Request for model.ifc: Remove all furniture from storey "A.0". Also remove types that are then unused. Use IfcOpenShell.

First a look at what the model holds.

```python
import ifcopenshell
import ifcopenshell.util.element

model = ifcopenshell.open("model.ifc")
print(model.schema)
storey = next(s for s in model.by_type("IfcBuildingStorey") if s.Name == "A.0")
furniture = [e for e in ifcopenshell.util.element.get_decomposition(storey) if e.is_a("IfcFurnishingElement")]
seen = {}
for e in furniture:
    element_type = ifcopenshell.util.element.get_type(e)
    name = element_type.Name if element_type not in (None, e) else None
    seen[name] = seen.get(name, 0) + 1
for name, count in sorted(seen.items(), key=str):
    print(count, "x", name)
```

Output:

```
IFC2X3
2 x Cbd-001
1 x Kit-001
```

```python
import ifcopenshell
import ifcopenshell.api.root
import ifcopenshell.util.element

model = ifcopenshell.open("model.ifc")

storey = next(s for s in model.by_type("IfcBuildingStorey") if s.Name == "A.0")
furniture = [e for e in ifcopenshell.util.element.get_decomposition(storey) if e.is_a("IfcFurnishingElement")]
types = {ifcopenshell.util.element.get_type(e) for e in furniture} - {None, *furniture}

for e in furniture:
    ifcopenshell.api.root.remove_product(model, product=e)
print(len(furniture), "removed")

unused = [t for t in types if not ifcopenshell.util.element.get_types(t)]
for t in unused:
    ifcopenshell.api.root.remove_product(model, product=t)
print(len(unused), "unused types removed")

model.write("model_updated.ifc")
```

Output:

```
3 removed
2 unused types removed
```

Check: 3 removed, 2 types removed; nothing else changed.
